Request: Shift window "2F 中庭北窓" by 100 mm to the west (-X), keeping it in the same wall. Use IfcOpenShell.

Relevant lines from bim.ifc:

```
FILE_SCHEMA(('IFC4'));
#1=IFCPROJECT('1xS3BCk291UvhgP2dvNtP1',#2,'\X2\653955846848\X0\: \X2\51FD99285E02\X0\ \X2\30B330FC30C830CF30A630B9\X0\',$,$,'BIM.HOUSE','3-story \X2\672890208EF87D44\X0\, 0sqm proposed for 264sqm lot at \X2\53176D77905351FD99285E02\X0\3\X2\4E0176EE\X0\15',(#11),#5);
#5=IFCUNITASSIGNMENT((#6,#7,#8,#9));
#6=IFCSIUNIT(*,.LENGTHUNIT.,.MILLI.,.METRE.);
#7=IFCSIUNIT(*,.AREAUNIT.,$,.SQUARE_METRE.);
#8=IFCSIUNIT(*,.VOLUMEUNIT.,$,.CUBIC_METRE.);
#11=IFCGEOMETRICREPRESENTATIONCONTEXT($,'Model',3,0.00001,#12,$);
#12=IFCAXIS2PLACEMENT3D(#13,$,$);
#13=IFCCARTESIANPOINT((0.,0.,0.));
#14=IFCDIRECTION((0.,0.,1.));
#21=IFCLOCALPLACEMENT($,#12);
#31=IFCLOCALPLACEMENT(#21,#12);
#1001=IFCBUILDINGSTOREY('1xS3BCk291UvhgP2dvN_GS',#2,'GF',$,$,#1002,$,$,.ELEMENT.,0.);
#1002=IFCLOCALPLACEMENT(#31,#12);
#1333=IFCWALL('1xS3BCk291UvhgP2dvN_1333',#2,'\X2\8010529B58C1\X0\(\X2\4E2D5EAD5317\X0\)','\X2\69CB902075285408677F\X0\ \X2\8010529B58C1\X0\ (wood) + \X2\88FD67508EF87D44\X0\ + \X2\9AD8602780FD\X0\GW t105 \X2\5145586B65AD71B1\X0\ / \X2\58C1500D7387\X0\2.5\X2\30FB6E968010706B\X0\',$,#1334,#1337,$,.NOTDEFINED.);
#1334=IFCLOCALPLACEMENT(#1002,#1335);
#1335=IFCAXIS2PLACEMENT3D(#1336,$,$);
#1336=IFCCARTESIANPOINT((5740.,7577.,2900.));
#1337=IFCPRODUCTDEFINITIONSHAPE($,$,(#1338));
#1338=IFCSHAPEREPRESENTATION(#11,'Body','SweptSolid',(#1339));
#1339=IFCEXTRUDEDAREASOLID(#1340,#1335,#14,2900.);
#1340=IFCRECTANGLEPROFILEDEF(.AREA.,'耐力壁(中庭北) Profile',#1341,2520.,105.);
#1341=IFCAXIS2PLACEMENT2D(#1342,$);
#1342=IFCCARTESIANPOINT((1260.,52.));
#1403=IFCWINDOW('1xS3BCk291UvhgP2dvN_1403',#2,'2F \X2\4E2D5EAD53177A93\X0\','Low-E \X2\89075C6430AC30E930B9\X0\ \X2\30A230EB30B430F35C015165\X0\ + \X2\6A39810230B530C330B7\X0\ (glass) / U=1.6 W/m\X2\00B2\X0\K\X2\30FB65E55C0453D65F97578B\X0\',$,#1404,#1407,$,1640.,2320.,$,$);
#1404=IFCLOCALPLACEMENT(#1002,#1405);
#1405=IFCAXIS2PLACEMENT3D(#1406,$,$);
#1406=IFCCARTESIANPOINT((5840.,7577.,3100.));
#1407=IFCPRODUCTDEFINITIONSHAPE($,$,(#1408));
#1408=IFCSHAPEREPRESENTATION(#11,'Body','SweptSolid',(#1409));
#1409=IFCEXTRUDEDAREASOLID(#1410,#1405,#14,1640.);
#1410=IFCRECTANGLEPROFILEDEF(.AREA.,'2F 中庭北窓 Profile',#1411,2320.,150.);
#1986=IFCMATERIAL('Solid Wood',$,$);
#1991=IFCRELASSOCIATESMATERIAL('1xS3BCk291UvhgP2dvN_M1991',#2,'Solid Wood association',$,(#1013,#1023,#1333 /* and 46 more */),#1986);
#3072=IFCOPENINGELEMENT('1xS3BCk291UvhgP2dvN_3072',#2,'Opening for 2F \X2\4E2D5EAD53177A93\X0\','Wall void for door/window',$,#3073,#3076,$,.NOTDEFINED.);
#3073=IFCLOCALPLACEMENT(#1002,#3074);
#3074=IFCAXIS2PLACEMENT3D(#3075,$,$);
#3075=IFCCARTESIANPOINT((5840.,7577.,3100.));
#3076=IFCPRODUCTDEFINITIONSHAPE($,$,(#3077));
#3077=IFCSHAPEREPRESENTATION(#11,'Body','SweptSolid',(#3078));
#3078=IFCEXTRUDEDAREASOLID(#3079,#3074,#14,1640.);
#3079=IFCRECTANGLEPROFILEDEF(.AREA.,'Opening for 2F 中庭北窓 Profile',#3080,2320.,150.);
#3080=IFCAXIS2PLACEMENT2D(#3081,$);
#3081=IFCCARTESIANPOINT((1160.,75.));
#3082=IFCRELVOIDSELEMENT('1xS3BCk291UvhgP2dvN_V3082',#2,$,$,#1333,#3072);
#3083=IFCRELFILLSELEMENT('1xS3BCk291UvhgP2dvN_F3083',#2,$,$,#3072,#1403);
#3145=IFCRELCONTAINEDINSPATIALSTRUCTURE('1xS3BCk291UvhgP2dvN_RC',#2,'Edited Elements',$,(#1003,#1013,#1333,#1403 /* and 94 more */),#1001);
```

```python
import ifcopenshell
import ifcopenshell.api.geometry
import ifcopenshell.util.placement

model = ifcopenshell.open("bim.ifc")

window = model.by_guid("1xS3BCk291UvhgP2dvN_1403")
opening = window.FillsVoids[0].RelatingOpeningElement
wall = opening.VoidsElements[0].RelatingBuildingElement

wall_matrix = ifcopenshell.util.placement.get_local_placement(wall.ObjectPlacement)
shift = wall_matrix[:3, 0] * -100.0
before = ifcopenshell.util.placement.get_local_placement(window.ObjectPlacement)[:3, 3].copy()

# The window is not placed relative to its opening, so move both.
for product in (opening, window):
    matrix = ifcopenshell.util.placement.get_local_placement(product.ObjectPlacement)
    matrix[:3, 3] += shift
    ifcopenshell.api.geometry.edit_object_placement(model, product=product, matrix=matrix, is_si=False)

after = ifcopenshell.util.placement.get_local_placement(window.ObjectPlacement)[:3, 3]
print("window moved by", (after - before).round(3) + 0.0)

model.write("bim_updated.ifc")
```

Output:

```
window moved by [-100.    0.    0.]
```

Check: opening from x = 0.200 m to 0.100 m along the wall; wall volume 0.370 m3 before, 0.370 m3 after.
